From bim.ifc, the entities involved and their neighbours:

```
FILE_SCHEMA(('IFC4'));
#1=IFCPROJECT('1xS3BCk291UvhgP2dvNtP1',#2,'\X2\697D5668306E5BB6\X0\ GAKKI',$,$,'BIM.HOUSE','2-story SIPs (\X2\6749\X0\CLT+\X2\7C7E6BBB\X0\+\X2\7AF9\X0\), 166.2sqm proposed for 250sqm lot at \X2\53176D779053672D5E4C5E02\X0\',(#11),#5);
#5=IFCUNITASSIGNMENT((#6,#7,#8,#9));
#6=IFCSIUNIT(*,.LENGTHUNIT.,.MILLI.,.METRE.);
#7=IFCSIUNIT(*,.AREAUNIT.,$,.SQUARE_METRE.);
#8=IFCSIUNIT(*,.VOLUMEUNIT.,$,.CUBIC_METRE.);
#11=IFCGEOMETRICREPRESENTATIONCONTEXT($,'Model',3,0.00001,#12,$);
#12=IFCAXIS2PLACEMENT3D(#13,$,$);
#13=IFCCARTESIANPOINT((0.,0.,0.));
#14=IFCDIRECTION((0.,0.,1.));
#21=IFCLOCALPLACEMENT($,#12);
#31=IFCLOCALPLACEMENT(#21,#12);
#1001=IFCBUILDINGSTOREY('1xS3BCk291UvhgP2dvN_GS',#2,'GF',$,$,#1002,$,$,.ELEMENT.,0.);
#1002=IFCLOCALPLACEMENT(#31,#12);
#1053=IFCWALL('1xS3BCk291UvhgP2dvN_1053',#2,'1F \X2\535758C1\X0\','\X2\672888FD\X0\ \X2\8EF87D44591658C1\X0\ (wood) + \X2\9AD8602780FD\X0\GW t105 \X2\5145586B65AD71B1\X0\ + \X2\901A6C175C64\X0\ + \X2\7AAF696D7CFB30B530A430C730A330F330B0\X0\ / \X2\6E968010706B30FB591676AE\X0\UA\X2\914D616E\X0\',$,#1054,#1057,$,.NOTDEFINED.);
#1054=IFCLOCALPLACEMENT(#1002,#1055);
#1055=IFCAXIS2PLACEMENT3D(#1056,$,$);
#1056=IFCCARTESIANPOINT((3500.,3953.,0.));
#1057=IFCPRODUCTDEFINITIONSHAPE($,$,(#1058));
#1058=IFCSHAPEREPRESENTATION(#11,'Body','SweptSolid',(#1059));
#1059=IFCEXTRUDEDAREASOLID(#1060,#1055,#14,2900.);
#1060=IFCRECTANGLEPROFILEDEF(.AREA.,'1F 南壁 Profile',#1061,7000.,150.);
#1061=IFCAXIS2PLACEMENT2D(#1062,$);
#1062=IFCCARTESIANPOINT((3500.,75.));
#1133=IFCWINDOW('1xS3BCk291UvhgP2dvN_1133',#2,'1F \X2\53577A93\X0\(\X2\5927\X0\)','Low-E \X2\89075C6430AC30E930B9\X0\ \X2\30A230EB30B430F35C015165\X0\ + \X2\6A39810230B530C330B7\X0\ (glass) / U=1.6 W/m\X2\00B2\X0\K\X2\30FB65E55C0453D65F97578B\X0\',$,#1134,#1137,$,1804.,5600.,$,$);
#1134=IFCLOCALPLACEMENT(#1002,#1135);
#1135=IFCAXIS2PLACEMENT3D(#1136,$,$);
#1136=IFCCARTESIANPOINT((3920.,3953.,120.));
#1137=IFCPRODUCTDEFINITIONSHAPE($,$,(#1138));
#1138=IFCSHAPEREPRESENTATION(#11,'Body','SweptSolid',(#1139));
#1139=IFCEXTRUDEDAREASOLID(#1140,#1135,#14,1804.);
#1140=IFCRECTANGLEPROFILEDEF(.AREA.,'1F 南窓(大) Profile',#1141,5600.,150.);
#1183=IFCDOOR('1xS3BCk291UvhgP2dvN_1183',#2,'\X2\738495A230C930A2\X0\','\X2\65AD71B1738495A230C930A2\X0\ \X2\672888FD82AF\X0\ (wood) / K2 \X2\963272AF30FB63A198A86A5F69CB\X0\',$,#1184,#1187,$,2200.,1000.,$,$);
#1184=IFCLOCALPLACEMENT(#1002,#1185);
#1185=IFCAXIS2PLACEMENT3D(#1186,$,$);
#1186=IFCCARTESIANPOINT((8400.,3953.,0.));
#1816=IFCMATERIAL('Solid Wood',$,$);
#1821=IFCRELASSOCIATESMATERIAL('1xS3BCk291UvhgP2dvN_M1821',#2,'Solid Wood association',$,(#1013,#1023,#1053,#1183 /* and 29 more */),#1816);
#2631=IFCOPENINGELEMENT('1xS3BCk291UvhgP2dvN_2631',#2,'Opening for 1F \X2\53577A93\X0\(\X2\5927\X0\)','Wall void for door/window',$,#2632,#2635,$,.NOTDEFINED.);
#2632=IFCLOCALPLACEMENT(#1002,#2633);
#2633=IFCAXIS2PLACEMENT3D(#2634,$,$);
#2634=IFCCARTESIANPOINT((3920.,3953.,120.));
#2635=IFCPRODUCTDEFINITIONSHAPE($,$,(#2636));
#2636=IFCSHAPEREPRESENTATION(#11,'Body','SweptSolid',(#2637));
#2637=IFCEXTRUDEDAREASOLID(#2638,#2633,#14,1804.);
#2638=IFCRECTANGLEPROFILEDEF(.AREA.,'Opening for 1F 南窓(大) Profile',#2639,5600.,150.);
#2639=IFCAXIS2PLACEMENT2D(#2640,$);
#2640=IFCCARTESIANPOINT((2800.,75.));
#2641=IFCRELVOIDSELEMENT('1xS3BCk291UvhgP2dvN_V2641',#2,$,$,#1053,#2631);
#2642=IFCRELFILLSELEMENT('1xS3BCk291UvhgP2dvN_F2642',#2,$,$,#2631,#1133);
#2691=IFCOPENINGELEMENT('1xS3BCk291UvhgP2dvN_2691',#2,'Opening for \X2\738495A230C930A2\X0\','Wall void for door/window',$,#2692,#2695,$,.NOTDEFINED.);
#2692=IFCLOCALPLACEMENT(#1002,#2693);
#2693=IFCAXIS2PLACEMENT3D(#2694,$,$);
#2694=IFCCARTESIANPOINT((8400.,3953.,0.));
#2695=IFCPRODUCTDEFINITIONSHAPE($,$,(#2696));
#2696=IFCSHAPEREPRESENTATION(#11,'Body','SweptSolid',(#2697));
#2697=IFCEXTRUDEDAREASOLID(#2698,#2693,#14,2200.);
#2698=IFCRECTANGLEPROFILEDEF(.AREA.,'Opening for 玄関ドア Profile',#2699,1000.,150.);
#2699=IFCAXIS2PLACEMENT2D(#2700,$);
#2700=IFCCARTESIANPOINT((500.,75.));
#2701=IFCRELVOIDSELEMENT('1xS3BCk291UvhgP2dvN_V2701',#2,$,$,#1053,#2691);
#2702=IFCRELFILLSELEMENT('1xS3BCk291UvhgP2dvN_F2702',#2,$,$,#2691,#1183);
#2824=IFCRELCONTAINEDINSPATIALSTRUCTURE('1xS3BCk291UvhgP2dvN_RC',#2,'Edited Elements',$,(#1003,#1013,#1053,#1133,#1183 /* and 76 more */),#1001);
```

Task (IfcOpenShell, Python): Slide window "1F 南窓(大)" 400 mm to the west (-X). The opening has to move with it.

```python
import ifcopenshell
import ifcopenshell.api.geometry
import ifcopenshell.util.placement
import ifcopenshell.util.unit

model = ifcopenshell.open("bim.ifc")
unit_scale = ifcopenshell.util.unit.calculate_unit_scale(model)

window = model.by_guid("1xS3BCk291UvhgP2dvN_1133")
opening = window.FillsVoids[0].RelatingOpeningElement
wall = opening.VoidsElements[0].RelatingBuildingElement

wall_matrix = ifcopenshell.util.placement.get_local_placement(wall.ObjectPlacement)
shift = wall_matrix[:3, 0] * -0.4 / unit_scale
before = ifcopenshell.util.placement.get_local_placement(window.ObjectPlacement)[:3, 3].copy()

# The window is not placed relative to its opening, so move both.
for product in (opening, window):
    matrix = ifcopenshell.util.placement.get_local_placement(product.ObjectPlacement)
    matrix[:3, 3] += shift
    ifcopenshell.api.geometry.edit_object_placement(model, product=product, matrix=matrix, is_si=False)

after = ifcopenshell.util.placement.get_local_placement(window.ObjectPlacement)[:3, 3]
print("window moved by", (after - before).round(3) + 0.0)

model.write("bim_edited.ifc")
```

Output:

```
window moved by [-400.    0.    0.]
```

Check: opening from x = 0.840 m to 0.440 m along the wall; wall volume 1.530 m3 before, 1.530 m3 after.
